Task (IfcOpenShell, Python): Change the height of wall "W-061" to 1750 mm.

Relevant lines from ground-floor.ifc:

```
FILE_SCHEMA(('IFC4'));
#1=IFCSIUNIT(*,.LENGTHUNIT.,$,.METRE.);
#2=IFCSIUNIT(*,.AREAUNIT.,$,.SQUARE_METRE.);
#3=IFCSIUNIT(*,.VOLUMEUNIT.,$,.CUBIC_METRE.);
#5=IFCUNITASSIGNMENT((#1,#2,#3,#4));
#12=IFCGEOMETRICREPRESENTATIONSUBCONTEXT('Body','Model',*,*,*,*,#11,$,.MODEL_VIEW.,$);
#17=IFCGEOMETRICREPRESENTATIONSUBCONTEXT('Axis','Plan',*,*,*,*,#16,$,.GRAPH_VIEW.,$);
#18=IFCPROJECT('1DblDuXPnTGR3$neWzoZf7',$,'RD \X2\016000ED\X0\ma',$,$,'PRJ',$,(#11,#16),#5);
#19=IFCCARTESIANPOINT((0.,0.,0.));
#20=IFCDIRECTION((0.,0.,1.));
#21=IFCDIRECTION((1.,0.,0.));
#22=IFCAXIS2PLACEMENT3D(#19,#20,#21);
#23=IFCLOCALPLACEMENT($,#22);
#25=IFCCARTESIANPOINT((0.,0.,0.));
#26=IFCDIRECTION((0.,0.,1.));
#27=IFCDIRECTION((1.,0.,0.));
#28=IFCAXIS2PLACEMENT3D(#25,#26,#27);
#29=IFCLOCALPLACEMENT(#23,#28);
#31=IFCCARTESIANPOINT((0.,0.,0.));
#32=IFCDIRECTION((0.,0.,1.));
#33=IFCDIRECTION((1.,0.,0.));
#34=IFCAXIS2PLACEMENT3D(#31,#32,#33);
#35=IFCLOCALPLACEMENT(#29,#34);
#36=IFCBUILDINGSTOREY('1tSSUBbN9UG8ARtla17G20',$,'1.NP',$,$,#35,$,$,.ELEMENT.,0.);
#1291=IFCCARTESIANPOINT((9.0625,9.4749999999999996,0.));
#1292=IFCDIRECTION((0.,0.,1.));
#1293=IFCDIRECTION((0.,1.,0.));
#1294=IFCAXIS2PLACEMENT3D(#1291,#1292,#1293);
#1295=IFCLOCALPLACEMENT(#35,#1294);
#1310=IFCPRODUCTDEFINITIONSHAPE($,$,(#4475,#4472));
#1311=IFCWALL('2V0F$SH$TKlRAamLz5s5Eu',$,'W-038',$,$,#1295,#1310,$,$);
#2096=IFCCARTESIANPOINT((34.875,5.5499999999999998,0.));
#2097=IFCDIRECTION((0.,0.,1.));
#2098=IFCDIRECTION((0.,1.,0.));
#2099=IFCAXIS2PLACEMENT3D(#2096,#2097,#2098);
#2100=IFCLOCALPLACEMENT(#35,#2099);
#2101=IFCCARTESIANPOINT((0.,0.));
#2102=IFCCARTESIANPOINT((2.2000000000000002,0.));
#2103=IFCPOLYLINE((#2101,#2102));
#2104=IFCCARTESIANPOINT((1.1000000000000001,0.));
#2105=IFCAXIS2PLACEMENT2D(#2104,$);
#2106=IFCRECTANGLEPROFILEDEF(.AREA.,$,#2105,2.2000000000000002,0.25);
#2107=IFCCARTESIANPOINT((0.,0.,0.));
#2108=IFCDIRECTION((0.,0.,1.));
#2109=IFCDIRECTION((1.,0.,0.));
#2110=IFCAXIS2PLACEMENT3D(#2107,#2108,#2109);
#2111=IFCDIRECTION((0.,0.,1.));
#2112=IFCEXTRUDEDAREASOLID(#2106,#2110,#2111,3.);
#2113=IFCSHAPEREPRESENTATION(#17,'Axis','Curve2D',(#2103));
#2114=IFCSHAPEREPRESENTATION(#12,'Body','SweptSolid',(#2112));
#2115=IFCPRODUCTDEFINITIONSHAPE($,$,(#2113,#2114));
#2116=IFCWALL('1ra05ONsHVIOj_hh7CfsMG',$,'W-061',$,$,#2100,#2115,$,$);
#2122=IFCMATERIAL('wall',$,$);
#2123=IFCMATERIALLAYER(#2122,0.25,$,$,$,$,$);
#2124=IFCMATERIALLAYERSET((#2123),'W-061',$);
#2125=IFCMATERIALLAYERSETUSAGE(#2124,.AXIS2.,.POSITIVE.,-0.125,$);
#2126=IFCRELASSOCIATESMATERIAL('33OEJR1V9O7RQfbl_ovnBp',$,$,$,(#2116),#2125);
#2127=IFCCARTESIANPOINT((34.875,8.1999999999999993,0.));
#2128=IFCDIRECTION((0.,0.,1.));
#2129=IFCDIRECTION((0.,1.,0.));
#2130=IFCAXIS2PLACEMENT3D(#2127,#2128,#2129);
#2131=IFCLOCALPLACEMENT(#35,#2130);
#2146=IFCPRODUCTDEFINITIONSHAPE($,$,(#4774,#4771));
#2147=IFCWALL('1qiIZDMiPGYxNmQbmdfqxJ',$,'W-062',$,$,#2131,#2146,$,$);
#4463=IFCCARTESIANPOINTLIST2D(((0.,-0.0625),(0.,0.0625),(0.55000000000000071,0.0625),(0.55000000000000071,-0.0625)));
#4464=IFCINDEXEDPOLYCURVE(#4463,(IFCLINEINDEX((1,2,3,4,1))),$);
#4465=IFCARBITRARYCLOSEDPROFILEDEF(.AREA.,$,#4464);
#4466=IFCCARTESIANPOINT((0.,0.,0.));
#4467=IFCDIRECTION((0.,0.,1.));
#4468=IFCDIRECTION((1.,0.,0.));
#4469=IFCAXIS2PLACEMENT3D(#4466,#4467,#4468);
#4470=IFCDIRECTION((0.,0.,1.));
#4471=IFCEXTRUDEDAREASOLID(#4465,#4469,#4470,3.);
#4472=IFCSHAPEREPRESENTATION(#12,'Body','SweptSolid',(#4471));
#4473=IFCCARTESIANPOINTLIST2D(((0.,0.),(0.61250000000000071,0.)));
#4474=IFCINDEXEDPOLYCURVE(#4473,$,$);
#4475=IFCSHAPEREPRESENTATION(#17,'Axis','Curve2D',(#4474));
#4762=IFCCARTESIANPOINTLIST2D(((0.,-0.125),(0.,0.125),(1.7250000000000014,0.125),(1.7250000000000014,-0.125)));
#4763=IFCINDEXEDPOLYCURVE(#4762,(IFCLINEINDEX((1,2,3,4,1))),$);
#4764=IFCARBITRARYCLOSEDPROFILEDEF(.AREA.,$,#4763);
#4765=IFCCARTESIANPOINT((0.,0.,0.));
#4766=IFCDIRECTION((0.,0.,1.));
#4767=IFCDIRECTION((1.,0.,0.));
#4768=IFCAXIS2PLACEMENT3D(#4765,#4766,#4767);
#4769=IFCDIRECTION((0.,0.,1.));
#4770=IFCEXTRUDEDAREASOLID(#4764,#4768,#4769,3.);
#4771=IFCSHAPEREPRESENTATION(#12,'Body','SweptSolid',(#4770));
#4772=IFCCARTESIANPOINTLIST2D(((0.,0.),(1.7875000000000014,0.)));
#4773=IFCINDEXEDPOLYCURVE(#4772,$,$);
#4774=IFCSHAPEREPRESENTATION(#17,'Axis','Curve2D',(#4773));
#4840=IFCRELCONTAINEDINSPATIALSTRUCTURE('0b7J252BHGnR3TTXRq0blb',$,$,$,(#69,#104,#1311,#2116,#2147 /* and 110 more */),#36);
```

```python
import ifcopenshell
import ifcopenshell.geom
import ifcopenshell.util.representation
import ifcopenshell.util.shape
import ifcopenshell.util.unit

model = ifcopenshell.open("ground-floor.ifc")
unit_scale = ifcopenshell.util.unit.calculate_unit_scale(model)
settings = ifcopenshell.geom.settings()


def volume(element):
    """Net volume in cubic metres, openings subtracted."""
    shape = ifcopenshell.geom.create_shape(settings, element)
    return ifcopenshell.util.shape.get_volume(shape.geometry)


wall = model.by_id(2116)
before = volume(wall)

body = ifcopenshell.util.representation.get_representation(wall, "Model", "Body")
solid = body.Items[0]
old_height = solid.Depth
solid.Depth = 1.75 / unit_scale
after = volume(wall)

print(f"height {old_height:g} -> {solid.Depth:g}, volume {before:.3f} -> {after:.3f} m3")

model.write("ground-floor_v2.ifc")
```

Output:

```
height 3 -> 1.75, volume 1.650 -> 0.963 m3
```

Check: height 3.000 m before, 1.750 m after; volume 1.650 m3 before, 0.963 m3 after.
